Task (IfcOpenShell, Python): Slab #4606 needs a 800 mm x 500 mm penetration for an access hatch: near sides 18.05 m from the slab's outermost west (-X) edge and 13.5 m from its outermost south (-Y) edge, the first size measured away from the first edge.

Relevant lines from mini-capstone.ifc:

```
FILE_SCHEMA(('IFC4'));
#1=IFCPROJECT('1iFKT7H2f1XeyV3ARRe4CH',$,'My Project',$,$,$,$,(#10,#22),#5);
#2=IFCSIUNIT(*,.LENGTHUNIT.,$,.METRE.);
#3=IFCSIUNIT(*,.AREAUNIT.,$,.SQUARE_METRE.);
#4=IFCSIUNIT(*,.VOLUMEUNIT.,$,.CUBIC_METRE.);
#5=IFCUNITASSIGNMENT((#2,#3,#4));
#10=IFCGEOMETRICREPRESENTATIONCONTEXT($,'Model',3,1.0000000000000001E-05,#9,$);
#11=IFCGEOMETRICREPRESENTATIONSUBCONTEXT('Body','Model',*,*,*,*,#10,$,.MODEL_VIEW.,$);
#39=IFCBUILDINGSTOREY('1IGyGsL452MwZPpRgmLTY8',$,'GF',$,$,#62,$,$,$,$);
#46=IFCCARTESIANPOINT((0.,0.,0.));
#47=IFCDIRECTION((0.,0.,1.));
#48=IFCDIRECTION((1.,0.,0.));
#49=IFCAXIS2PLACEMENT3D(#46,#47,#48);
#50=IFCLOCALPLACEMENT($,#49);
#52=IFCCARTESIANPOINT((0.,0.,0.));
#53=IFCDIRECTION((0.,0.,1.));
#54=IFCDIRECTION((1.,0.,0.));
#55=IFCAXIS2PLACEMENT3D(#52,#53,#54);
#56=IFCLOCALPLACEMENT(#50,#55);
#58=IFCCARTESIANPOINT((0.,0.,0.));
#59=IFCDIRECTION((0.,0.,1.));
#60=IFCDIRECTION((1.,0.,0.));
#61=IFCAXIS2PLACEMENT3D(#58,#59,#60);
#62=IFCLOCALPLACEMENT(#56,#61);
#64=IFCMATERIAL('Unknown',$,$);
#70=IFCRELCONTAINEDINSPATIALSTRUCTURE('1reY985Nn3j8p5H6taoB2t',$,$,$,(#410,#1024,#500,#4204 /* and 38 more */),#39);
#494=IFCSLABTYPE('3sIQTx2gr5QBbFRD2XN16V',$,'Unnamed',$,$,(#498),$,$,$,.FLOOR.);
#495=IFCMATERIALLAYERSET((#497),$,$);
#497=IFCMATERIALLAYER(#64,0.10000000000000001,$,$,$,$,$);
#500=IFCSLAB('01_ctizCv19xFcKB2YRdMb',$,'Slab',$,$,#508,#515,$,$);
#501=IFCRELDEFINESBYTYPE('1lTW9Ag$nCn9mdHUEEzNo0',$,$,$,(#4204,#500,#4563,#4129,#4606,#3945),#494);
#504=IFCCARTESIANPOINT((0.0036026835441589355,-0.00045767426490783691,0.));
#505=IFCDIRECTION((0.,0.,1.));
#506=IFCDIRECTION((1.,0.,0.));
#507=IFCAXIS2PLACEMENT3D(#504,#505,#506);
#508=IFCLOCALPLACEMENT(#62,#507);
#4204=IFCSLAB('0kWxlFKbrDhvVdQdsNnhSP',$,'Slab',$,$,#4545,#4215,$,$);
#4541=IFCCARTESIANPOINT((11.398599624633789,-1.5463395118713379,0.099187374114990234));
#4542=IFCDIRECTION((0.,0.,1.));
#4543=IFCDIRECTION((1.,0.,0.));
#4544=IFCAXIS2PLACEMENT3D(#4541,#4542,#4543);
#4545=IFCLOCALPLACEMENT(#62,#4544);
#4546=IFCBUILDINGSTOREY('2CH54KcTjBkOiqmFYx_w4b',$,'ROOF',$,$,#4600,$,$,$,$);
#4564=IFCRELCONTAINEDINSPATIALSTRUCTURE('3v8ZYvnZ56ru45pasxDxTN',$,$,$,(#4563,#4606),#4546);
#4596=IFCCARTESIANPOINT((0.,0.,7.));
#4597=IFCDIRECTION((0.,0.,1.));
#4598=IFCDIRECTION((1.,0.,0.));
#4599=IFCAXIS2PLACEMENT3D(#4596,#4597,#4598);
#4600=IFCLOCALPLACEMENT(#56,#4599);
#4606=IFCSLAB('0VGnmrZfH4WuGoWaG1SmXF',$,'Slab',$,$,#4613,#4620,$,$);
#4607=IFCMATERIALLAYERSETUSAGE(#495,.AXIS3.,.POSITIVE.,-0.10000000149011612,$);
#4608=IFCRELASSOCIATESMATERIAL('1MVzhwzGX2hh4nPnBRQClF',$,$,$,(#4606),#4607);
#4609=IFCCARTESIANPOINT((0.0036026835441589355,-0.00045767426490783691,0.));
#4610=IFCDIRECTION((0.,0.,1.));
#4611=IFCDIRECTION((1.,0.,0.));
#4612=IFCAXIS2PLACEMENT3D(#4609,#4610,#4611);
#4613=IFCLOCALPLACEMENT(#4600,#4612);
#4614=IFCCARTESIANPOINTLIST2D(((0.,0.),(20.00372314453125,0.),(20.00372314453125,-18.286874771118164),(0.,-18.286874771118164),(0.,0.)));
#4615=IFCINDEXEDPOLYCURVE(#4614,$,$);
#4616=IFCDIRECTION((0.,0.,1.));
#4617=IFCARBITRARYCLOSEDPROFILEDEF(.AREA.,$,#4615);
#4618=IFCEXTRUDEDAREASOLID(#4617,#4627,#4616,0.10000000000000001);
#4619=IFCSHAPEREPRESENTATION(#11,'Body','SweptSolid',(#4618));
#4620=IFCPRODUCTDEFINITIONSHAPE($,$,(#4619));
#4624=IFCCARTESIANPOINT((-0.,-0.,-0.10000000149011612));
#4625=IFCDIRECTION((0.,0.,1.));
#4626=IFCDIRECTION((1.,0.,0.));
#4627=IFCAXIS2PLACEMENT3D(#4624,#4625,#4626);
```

```python
import numpy as np
import ifcopenshell
import ifcopenshell.api.feature
import ifcopenshell.api.geometry
import ifcopenshell.api.root
import ifcopenshell.geom
import ifcopenshell.util.placement
import ifcopenshell.util.representation
import ifcopenshell.util.shape
import ifcopenshell.util.unit

model = ifcopenshell.open("mini-capstone.ifc")
unit_scale = ifcopenshell.util.unit.calculate_unit_scale(model)
settings = ifcopenshell.geom.settings()


def volume(element):
    """Net volume in cubic metres, openings subtracted."""
    shape = ifcopenshell.geom.create_shape(settings, element)
    return ifcopenshell.util.shape.get_volume(shape.geometry)


slab = model.by_guid("0VGnmrZfH4WuGoWaG1SmXF")
before = volume(slab)

# Extent in the slab's own axes, in metres. The edges named are its -X and -Y sides.
slab_shape = ifcopenshell.geom.create_shape(settings, slab)
vertices = ifcopenshell.util.shape.get_vertices(slab_shape.geometry)
x_min, y_min, bottom = vertices.min(axis=0)
top = vertices[:, 2].max()

opening = ifcopenshell.api.root.create_entity(model, ifc_class="IfcOpeningElement", name="Access hatch opening", predefined_type="OPENING")
context = ifcopenshell.util.representation.get_context(model, "Model", "Body", "MODEL_VIEW")
width, depth = 0.8, 0.5
outline = [(0.0, 0.0), (width, 0.0), (width, depth), (0.0, depth), (0.0, 0.0)]
# Overshoot both faces by 50 mm so the cut is clean.
shape = ifcopenshell.api.geometry.add_slab_representation(
    model, context=context, depth=top - bottom + 0.1, polyline=outline
)
ifcopenshell.api.geometry.assign_representation(model, product=opening, representation=shape)

matrix = ifcopenshell.util.placement.get_local_placement(slab.ObjectPlacement)
matrix[:, 3] = matrix @ np.append(np.array([x_min + 18.05, y_min + 13.5, bottom - 0.05]) / unit_scale, 1.0)
ifcopenshell.api.geometry.edit_object_placement(model, product=opening, matrix=matrix, is_si=False)
ifcopenshell.api.feature.add_feature(model, feature=opening, element=slab)

after = volume(slab)

print(f"slab volume {before:.3f} -> {after:.3f} m3")

model.write("mini-capstone-out.ifc")
```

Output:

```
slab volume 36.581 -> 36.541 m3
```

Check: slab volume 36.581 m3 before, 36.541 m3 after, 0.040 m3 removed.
